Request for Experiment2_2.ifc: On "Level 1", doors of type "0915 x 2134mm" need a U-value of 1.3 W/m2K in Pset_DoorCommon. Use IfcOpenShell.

First a look at what the model holds.

```python
import ifcopenshell
import ifcopenshell.util.element

model = ifcopenshell.open("Experiment2_2.ifc")
print(model.schema)
storey = next(s for s in model.by_type("IfcBuildingStorey") if s.Name == "Level 1")
doors = [e for e in ifcopenshell.util.element.get_decomposition(storey) if e.is_a("IfcDoor")]
seen = {}
for e in doors:
    element_type = ifcopenshell.util.element.get_type(e)
    key = (element_type.Name if element_type != e and element_type else None, ifcopenshell.util.element.get_pset(e, "Pset_DoorCommon", "ThermalTransmittance"))
    seen[key] = seen.get(key, 0) + 1
for (name, value), count in sorted(seen.items(), key=str):
    print(count, "x", name, "|", value)
```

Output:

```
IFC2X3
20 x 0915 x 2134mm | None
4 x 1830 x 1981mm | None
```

```python
import ifcopenshell
import ifcopenshell.api.pset
import ifcopenshell.util.element

model = ifcopenshell.open("Experiment2_2.ifc")

storey = next(s for s in model.by_type("IfcBuildingStorey") if s.Name == "Level 1")
doors = [e for e in ifcopenshell.util.element.get_decomposition(storey) if e.is_a("IfcDoor")]

count = 0
for e in doors:
    element_type = ifcopenshell.util.element.get_type(e)
    if element_type in (None, e) or element_type.Name != "0915 x 2134mm":
        continue
    # add_pset returns the element's existing set when there is one.
    pset = ifcopenshell.api.pset.add_pset(model, product=e, name="Pset_DoorCommon")
    ifcopenshell.api.pset.edit_pset(model, pset=pset, properties={"ThermalTransmittance": 1.3})
    count += 1

print(count, "doors updated")

model.write("Experiment2_2_updated.ifc")
```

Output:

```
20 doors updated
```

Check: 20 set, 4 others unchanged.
